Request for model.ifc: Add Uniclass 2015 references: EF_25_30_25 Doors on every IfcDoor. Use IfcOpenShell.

First a look at what the model holds.

```python
import ifcopenshell

model = ifcopenshell.open("model.ifc")
print(model.schema)
print("classifications:", [c.Name for c in model.by_type("IfcClassification")])
for ifc_class in ("IfcDoor", "IfcRoof", "IfcStair", "IfcWall", "IfcWindow"):
    print(ifc_class, len(model.by_type(ifc_class)))
```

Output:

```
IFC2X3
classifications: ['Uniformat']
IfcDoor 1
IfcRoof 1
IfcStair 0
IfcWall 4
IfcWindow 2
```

```python
import ifcopenshell
import ifcopenshell.api.classification

model = ifcopenshell.open("model.ifc")

# IFC2X3 requires Source and Edition and has no link from the project to the system.
system = model.create_entity("IfcClassification", Source="NBS", Edition="2015", Name="Uniclass 2015")

codes = {
    "IfcDoor": ("EF_25_30_25", "Doors"),
}
for ifc_class, (code, name) in codes.items():
    products = model.by_type(ifc_class)
    ifcopenshell.api.classification.add_reference(
        model, products=products, classification=system, identification=code, name=name
    )
    print(code, len(products))

model.write("model_v2.ifc")
```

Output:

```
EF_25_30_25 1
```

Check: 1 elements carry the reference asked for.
